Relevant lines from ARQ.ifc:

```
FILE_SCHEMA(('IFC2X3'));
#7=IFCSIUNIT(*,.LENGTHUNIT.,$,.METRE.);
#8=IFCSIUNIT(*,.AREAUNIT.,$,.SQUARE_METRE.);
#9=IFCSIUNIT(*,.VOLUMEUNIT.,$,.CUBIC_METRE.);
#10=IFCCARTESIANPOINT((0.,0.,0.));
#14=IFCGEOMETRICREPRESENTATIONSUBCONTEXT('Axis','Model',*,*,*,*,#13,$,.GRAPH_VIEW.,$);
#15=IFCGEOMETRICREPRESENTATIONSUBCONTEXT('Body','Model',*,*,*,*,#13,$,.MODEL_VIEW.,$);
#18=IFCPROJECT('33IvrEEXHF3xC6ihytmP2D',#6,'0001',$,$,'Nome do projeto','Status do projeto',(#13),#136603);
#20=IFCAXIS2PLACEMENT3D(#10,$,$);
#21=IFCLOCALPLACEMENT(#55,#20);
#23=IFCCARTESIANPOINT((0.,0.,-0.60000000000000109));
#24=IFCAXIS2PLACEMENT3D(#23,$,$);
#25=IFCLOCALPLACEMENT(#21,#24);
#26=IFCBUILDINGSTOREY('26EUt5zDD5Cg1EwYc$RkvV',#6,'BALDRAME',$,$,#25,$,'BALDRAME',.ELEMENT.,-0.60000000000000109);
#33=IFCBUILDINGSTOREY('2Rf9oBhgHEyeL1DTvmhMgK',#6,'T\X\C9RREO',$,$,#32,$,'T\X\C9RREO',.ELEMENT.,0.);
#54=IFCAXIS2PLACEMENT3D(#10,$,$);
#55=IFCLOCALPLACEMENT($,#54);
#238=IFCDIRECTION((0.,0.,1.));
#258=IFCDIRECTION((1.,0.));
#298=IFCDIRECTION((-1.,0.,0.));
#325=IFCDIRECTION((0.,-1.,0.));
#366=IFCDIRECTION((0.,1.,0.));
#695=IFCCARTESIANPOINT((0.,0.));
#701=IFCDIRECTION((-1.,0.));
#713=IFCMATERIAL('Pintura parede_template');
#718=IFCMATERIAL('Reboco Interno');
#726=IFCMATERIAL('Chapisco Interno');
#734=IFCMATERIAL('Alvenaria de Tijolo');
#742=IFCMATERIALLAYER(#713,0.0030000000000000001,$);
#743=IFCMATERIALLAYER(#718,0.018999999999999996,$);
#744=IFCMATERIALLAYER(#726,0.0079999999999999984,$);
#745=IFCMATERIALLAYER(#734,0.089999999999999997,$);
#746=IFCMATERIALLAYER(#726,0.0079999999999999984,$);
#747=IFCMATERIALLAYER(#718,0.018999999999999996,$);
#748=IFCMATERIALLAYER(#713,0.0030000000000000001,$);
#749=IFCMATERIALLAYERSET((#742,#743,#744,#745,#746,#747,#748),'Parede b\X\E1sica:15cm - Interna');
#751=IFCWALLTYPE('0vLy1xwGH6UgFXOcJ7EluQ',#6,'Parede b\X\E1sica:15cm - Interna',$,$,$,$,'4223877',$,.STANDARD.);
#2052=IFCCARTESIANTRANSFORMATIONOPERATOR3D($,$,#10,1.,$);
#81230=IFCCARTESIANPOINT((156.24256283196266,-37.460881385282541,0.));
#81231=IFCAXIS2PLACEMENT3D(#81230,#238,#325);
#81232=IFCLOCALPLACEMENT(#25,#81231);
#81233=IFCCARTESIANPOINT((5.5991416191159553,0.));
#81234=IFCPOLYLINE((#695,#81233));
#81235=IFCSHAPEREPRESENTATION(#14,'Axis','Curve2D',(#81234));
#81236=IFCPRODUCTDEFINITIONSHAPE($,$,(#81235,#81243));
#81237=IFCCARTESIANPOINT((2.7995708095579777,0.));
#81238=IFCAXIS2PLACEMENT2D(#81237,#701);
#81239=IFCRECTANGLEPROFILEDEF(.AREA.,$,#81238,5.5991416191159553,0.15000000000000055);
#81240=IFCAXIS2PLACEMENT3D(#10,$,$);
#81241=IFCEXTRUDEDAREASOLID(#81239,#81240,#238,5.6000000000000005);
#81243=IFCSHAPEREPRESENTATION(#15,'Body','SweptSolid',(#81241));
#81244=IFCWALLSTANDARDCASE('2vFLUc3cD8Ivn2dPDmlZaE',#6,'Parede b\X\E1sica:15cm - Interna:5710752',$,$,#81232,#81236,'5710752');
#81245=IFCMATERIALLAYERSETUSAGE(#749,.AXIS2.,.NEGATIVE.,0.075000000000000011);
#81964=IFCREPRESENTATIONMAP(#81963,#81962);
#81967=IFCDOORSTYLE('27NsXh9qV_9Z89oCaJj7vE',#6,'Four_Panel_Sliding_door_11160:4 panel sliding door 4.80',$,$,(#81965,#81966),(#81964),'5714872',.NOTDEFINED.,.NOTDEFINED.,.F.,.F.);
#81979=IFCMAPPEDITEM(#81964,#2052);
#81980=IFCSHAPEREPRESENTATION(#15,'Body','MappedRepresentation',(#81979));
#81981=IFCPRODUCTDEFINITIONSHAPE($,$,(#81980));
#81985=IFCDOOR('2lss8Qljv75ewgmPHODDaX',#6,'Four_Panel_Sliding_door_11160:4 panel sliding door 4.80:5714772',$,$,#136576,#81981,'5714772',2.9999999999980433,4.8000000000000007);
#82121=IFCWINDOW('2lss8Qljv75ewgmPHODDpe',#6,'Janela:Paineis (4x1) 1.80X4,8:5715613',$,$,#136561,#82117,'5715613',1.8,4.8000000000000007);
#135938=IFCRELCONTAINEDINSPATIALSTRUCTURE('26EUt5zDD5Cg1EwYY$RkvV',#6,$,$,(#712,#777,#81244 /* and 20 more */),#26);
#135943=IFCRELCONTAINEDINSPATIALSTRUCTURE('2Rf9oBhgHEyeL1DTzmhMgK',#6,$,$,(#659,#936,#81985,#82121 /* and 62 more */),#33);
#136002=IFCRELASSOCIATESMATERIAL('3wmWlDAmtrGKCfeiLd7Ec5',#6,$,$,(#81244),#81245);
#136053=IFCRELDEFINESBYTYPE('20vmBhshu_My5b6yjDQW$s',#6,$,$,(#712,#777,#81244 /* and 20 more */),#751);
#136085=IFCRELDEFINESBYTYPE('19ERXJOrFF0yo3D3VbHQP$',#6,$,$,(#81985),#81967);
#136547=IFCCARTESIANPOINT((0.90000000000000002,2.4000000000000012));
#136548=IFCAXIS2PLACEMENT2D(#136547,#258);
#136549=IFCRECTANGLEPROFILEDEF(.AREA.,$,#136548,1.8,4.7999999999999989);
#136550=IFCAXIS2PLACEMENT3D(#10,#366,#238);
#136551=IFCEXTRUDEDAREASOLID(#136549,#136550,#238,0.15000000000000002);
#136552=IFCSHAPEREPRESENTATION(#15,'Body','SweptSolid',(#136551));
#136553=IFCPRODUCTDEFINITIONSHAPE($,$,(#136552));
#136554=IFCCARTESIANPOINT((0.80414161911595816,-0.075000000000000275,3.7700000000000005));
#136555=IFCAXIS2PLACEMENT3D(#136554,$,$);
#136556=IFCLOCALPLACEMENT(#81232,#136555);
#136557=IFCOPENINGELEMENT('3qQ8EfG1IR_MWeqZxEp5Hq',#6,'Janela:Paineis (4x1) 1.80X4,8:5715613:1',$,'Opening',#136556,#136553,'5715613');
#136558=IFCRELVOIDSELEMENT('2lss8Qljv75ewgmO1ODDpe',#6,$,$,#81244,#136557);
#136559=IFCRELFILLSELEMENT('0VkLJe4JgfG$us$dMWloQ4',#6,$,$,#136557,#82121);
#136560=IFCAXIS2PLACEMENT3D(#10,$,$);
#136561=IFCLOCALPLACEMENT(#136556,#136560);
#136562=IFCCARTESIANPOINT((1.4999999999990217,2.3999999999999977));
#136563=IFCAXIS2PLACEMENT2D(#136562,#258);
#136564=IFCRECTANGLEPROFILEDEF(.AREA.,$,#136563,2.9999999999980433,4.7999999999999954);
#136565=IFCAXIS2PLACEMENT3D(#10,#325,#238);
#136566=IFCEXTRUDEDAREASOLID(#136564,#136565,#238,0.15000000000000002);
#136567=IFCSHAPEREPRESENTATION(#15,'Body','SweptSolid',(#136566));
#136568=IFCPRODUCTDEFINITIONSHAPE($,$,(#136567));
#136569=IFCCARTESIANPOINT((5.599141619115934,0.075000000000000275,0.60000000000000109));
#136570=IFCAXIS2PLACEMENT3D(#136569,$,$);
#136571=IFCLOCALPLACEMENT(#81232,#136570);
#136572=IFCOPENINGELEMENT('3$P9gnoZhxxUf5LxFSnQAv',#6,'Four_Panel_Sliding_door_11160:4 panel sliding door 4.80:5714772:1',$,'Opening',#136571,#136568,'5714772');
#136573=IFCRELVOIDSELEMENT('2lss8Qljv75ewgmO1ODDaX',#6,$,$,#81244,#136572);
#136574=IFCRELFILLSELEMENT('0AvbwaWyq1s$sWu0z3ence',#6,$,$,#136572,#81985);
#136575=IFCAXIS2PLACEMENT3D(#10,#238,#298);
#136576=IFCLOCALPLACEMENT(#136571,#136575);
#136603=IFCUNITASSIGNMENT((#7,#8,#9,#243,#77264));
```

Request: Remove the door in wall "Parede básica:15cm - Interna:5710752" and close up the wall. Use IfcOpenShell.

```python
import ifcopenshell
import ifcopenshell.api.feature
import ifcopenshell.api.root
import ifcopenshell.geom
import ifcopenshell.util.shape

model = ifcopenshell.open("ARQ.ifc")
settings = ifcopenshell.geom.settings()


def volume(element):
    """Net volume in cubic metres, openings subtracted."""
    shape = ifcopenshell.geom.create_shape(settings, element)
    return ifcopenshell.util.shape.get_volume(shape.geometry)


door = model.by_guid("2lss8Qljv75ewgmPHODDaX")
opening = door.FillsVoids[0].RelatingOpeningElement
wall = opening.VoidsElements[0].RelatingBuildingElement
before = volume(wall)

ifcopenshell.api.root.remove_product(model, product=door)
ifcopenshell.api.feature.remove_feature(model, feature=opening)

after = volume(wall)

print(f"wall volume {before:.3f} -> {after:.3f} m3")

model.write("ARQ-out.ifc")
```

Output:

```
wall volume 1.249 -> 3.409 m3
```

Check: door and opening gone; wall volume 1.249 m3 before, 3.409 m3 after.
